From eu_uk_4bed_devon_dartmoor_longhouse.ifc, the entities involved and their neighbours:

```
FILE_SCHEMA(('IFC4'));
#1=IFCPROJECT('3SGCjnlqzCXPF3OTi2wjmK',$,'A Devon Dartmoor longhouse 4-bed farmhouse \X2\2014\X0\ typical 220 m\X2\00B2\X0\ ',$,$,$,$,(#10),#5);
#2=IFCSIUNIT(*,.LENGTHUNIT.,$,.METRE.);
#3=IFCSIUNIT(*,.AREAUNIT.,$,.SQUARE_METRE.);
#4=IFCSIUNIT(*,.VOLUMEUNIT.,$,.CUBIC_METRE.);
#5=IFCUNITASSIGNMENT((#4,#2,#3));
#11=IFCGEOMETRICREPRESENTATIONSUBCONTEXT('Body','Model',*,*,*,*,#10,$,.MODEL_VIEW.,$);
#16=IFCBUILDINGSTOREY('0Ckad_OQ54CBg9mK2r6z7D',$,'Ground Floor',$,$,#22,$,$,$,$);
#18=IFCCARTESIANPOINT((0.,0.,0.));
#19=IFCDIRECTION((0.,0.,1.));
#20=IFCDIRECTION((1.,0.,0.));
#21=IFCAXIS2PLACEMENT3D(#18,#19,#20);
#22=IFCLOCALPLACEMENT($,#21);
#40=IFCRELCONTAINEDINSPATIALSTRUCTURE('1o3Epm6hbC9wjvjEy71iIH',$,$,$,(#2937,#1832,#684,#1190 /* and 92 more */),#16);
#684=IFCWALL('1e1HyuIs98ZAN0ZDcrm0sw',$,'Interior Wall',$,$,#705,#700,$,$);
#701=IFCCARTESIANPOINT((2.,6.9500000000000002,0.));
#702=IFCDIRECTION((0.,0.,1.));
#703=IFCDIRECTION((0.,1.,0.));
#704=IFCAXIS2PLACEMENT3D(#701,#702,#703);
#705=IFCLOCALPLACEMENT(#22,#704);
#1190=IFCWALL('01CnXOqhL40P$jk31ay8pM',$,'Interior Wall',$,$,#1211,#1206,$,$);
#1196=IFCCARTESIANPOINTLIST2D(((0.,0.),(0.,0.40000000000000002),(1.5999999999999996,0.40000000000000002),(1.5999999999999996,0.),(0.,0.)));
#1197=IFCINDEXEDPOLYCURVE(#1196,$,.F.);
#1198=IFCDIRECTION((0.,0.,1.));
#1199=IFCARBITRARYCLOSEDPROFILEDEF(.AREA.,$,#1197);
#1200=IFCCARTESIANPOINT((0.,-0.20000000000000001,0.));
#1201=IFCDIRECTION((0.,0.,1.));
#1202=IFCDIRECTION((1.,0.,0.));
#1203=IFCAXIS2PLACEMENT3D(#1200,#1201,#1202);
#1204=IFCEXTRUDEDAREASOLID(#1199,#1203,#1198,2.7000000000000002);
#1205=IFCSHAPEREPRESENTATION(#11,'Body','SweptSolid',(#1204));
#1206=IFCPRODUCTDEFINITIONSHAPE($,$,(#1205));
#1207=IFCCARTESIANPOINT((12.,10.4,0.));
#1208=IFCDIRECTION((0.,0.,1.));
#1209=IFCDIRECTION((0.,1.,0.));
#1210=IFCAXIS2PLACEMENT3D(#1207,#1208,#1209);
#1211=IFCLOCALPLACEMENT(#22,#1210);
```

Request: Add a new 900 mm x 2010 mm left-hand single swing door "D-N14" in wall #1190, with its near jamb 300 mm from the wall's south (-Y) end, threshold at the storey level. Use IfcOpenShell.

```python
import numpy as np
import ifcopenshell
import ifcopenshell.api.feature
import ifcopenshell.api.geometry
import ifcopenshell.api.root
import ifcopenshell.api.spatial
import ifcopenshell.geom
import ifcopenshell.util.element
import ifcopenshell.util.placement
import ifcopenshell.util.representation
import ifcopenshell.util.shape
import ifcopenshell.util.unit

model = ifcopenshell.open("eu_uk_4bed_devon_dartmoor_longhouse.ifc")
unit_scale = ifcopenshell.util.unit.calculate_unit_scale(model)
settings = ifcopenshell.geom.settings()


def volume(element):
    """Net volume in cubic metres, openings subtracted."""
    shape = ifcopenshell.geom.create_shape(settings, element)
    return ifcopenshell.util.shape.get_volume(shape.geometry)


wall = model.by_guid("01CnXOqhL40P$jk31ay8pM")
storey = ifcopenshell.util.element.get_container(wall, ifc_class="IfcBuildingStorey")
context = ifcopenshell.util.representation.get_context(model, "Model", "Body", "MODEL_VIEW")
before = volume(wall)

width, height, from_end, sill = 0.9, 2.01, 0.3, 0.0  # metres

# The wall runs along its own X axis, and the end named is its -X end.
wall_shape = ifcopenshell.geom.create_shape(settings, wall)
x, y, z = ifcopenshell.util.shape.get_vertices(wall_shape.geometry).T
start = x.min() + from_end
face, thickness = float(y.min()), float(y.max() - y.min())
wall_matrix = ifcopenshell.util.placement.get_local_placement(wall.ObjectPlacement)
level = ifcopenshell.util.placement.get_local_placement(storey.ObjectPlacement)[2, 3]


def in_wall(x, y):
    """Placement at x, y metres in the wall's axes, at sill height."""
    matrix = wall_matrix.copy()
    matrix[:, 3] = wall_matrix @ np.array([x / unit_scale, y / unit_scale, 0.0, 1.0])
    matrix[2, 3] = level + sill / unit_scale
    return matrix


# Opening: a box that overshoots both wall faces by 50 mm.
opening = ifcopenshell.api.root.create_entity(model, ifc_class="IfcOpeningElement", predefined_type="OPENING")
box = ifcopenshell.api.geometry.add_wall_representation(
    model, context=context, length=width, height=height, thickness=thickness + 0.1
)
ifcopenshell.api.geometry.assign_representation(model, product=opening, representation=box)
ifcopenshell.api.geometry.edit_object_placement(model, product=opening, matrix=in_wall(start, face - 0.05), is_si=False)
ifcopenshell.api.feature.add_feature(model, feature=opening, element=wall)

door = ifcopenshell.api.root.create_entity(model, ifc_class="IfcDoor", name="D-N14", predefined_type="DOOR")
door.OverallWidth, door.OverallHeight = width / unit_scale, height / unit_scale
door.OperationType = "SINGLE_SWING_LEFT"
body = ifcopenshell.api.geometry.add_door_representation(
    model,
    context=context,
    overall_width=door.OverallWidth,
    overall_height=door.OverallHeight,
    operation_type="SINGLE_SWING_LEFT",
    lining_properties={"LiningDepth": thickness / unit_scale, "ThresholdDepth": thickness / unit_scale},
)
ifcopenshell.api.geometry.assign_representation(model, product=door, representation=body)
ifcopenshell.api.spatial.assign_container(model, products=[door], relating_structure=storey)
ifcopenshell.api.feature.add_filling(model, opening=opening, element=door)

# The lining spans the wall, so the door starts at the wall face.
ifcopenshell.api.geometry.edit_object_placement(model, product=door, matrix=in_wall(start, face), is_si=False)

after = volume(wall)

print(f"wall volume {before:.3f} -> {after:.3f} m3")

model.write("eu_uk_4bed_devon_dartmoor_longhouse-out.ifc")
```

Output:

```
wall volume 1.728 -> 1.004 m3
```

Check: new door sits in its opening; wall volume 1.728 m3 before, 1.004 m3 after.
